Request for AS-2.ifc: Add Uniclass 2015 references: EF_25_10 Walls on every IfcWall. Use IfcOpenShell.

First a look at what the model holds.

```python
import ifcopenshell

model = ifcopenshell.open("AS-2.ifc")
print(model.schema)
print("classifications:", [c.Name for c in model.by_type("IfcClassification")])
for ifc_class in ("IfcDoor", "IfcRoof", "IfcStair", "IfcWall", "IfcWindow"):
    print(ifc_class, len(model.by_type(ifc_class)))
```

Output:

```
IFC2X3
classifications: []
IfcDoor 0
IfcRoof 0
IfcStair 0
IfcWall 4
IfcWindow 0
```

```python
import ifcopenshell
import ifcopenshell.api.classification

model = ifcopenshell.open("AS-2.ifc")

# IFC2X3 requires Source and Edition and has no link from the project to the system.
system = model.create_entity("IfcClassification", Source="NBS", Edition="2015", Name="Uniclass 2015")

codes = {
    "IfcWall": ("EF_25_10", "Walls"),
}
for ifc_class, (code, name) in codes.items():
    products = model.by_type(ifc_class)
    ifcopenshell.api.classification.add_reference(
        model, products=products, classification=system, identification=code, name=name
    )
    print(code, len(products))

model.write("AS-2-out.ifc")
```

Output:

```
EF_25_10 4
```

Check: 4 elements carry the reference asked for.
